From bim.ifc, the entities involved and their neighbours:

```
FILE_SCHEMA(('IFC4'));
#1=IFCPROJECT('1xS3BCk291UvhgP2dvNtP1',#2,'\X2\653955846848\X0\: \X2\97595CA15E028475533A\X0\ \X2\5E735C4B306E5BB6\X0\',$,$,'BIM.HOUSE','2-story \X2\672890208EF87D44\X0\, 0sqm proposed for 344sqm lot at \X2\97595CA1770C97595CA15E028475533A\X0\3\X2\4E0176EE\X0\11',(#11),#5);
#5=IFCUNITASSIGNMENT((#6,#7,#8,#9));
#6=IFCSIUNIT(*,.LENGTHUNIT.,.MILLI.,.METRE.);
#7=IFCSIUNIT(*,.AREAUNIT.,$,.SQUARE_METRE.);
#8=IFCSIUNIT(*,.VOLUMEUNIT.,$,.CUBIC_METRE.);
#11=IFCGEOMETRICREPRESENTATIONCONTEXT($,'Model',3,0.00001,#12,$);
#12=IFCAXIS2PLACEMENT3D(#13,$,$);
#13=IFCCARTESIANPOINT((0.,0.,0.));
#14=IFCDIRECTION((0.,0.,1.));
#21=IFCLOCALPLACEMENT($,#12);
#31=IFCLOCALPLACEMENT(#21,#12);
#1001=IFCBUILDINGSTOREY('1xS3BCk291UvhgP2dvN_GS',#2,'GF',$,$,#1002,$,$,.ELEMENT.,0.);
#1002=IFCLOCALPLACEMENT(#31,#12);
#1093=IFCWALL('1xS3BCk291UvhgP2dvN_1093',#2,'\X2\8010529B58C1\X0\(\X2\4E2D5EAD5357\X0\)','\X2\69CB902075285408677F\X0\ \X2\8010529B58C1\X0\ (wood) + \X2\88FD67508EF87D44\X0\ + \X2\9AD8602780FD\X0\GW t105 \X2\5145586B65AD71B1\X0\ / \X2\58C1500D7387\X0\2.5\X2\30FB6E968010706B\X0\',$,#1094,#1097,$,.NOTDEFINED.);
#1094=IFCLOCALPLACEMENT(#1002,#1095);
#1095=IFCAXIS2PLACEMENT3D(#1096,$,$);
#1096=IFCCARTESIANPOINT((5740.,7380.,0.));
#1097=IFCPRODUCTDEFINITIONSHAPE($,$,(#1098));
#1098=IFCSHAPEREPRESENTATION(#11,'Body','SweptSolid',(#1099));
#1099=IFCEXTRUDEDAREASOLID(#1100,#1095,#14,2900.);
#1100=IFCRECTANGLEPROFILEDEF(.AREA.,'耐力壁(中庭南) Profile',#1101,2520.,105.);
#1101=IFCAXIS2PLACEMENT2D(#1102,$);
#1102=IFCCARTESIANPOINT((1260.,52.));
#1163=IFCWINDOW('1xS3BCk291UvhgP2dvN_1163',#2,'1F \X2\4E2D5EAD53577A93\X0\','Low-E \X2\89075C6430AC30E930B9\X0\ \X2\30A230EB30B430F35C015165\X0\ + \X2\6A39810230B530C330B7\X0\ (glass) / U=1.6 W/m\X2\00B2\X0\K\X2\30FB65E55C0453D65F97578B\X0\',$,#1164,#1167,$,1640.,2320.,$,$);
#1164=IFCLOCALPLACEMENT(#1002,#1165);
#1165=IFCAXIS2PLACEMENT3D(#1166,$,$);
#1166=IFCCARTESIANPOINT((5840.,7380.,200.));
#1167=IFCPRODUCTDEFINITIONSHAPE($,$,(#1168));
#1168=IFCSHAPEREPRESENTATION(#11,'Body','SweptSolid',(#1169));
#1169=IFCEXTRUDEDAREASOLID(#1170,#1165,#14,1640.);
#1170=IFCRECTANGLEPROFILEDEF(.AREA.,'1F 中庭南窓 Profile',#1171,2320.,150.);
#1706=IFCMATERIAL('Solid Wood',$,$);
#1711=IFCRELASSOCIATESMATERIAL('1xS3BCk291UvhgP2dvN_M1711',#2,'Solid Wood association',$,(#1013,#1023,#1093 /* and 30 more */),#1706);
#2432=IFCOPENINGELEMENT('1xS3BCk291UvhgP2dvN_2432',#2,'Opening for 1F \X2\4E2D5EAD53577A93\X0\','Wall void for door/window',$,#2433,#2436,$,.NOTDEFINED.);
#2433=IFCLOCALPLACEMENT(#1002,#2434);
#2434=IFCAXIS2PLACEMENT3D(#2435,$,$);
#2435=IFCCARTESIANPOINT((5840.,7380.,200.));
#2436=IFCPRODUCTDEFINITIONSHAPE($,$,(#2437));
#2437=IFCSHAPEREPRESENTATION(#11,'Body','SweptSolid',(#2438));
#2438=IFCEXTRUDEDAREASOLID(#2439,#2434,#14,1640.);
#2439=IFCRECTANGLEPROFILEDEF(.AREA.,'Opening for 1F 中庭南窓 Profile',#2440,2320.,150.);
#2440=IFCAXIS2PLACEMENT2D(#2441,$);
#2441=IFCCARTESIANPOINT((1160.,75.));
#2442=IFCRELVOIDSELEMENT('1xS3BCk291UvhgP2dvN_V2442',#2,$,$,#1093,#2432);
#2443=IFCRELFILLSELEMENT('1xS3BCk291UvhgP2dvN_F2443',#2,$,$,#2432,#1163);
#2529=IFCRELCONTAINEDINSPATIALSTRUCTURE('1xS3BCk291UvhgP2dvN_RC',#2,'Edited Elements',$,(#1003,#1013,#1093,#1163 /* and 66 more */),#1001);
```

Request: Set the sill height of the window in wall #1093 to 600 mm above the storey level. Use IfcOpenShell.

```python
import numpy as np
import ifcopenshell
import ifcopenshell.api.geometry
import ifcopenshell.geom
import ifcopenshell.util.element
import ifcopenshell.util.placement
import ifcopenshell.util.shape
import ifcopenshell.util.unit

model = ifcopenshell.open("bim.ifc")
unit_scale = ifcopenshell.util.unit.calculate_unit_scale(model)

window = model.by_id(1163)
opening = window.FillsVoids[0].RelatingOpeningElement
storey = ifcopenshell.util.element.get_container(window, ifc_class="IfcBuildingStorey")
level = ifcopenshell.util.placement.get_local_placement(storey.ObjectPlacement)[2, 3]

# The opening's origin need not be at the sill, so measure its lowest point.
shape = ifcopenshell.geom.create_shape(ifcopenshell.geom.settings(), opening)
bottom = ifcopenshell.util.shape.get_shape_bottom_elevation(shape, shape.geometry) / unit_scale
dz = level + 0.6 / unit_scale - bottom

shift = np.array([0.0, 0.0, dz])
# The window is not placed relative to its opening, so move both.
for product in (opening, window):
    matrix = ifcopenshell.util.placement.get_local_placement(product.ObjectPlacement)
    matrix[:3, 3] += shift
    ifcopenshell.api.geometry.edit_object_placement(model, product=product, matrix=matrix, is_si=False)

print(f"moved by {dz * unit_scale:+.3f} m")

model.write("bim_updated.ifc")
```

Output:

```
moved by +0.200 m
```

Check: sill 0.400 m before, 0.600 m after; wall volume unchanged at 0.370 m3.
